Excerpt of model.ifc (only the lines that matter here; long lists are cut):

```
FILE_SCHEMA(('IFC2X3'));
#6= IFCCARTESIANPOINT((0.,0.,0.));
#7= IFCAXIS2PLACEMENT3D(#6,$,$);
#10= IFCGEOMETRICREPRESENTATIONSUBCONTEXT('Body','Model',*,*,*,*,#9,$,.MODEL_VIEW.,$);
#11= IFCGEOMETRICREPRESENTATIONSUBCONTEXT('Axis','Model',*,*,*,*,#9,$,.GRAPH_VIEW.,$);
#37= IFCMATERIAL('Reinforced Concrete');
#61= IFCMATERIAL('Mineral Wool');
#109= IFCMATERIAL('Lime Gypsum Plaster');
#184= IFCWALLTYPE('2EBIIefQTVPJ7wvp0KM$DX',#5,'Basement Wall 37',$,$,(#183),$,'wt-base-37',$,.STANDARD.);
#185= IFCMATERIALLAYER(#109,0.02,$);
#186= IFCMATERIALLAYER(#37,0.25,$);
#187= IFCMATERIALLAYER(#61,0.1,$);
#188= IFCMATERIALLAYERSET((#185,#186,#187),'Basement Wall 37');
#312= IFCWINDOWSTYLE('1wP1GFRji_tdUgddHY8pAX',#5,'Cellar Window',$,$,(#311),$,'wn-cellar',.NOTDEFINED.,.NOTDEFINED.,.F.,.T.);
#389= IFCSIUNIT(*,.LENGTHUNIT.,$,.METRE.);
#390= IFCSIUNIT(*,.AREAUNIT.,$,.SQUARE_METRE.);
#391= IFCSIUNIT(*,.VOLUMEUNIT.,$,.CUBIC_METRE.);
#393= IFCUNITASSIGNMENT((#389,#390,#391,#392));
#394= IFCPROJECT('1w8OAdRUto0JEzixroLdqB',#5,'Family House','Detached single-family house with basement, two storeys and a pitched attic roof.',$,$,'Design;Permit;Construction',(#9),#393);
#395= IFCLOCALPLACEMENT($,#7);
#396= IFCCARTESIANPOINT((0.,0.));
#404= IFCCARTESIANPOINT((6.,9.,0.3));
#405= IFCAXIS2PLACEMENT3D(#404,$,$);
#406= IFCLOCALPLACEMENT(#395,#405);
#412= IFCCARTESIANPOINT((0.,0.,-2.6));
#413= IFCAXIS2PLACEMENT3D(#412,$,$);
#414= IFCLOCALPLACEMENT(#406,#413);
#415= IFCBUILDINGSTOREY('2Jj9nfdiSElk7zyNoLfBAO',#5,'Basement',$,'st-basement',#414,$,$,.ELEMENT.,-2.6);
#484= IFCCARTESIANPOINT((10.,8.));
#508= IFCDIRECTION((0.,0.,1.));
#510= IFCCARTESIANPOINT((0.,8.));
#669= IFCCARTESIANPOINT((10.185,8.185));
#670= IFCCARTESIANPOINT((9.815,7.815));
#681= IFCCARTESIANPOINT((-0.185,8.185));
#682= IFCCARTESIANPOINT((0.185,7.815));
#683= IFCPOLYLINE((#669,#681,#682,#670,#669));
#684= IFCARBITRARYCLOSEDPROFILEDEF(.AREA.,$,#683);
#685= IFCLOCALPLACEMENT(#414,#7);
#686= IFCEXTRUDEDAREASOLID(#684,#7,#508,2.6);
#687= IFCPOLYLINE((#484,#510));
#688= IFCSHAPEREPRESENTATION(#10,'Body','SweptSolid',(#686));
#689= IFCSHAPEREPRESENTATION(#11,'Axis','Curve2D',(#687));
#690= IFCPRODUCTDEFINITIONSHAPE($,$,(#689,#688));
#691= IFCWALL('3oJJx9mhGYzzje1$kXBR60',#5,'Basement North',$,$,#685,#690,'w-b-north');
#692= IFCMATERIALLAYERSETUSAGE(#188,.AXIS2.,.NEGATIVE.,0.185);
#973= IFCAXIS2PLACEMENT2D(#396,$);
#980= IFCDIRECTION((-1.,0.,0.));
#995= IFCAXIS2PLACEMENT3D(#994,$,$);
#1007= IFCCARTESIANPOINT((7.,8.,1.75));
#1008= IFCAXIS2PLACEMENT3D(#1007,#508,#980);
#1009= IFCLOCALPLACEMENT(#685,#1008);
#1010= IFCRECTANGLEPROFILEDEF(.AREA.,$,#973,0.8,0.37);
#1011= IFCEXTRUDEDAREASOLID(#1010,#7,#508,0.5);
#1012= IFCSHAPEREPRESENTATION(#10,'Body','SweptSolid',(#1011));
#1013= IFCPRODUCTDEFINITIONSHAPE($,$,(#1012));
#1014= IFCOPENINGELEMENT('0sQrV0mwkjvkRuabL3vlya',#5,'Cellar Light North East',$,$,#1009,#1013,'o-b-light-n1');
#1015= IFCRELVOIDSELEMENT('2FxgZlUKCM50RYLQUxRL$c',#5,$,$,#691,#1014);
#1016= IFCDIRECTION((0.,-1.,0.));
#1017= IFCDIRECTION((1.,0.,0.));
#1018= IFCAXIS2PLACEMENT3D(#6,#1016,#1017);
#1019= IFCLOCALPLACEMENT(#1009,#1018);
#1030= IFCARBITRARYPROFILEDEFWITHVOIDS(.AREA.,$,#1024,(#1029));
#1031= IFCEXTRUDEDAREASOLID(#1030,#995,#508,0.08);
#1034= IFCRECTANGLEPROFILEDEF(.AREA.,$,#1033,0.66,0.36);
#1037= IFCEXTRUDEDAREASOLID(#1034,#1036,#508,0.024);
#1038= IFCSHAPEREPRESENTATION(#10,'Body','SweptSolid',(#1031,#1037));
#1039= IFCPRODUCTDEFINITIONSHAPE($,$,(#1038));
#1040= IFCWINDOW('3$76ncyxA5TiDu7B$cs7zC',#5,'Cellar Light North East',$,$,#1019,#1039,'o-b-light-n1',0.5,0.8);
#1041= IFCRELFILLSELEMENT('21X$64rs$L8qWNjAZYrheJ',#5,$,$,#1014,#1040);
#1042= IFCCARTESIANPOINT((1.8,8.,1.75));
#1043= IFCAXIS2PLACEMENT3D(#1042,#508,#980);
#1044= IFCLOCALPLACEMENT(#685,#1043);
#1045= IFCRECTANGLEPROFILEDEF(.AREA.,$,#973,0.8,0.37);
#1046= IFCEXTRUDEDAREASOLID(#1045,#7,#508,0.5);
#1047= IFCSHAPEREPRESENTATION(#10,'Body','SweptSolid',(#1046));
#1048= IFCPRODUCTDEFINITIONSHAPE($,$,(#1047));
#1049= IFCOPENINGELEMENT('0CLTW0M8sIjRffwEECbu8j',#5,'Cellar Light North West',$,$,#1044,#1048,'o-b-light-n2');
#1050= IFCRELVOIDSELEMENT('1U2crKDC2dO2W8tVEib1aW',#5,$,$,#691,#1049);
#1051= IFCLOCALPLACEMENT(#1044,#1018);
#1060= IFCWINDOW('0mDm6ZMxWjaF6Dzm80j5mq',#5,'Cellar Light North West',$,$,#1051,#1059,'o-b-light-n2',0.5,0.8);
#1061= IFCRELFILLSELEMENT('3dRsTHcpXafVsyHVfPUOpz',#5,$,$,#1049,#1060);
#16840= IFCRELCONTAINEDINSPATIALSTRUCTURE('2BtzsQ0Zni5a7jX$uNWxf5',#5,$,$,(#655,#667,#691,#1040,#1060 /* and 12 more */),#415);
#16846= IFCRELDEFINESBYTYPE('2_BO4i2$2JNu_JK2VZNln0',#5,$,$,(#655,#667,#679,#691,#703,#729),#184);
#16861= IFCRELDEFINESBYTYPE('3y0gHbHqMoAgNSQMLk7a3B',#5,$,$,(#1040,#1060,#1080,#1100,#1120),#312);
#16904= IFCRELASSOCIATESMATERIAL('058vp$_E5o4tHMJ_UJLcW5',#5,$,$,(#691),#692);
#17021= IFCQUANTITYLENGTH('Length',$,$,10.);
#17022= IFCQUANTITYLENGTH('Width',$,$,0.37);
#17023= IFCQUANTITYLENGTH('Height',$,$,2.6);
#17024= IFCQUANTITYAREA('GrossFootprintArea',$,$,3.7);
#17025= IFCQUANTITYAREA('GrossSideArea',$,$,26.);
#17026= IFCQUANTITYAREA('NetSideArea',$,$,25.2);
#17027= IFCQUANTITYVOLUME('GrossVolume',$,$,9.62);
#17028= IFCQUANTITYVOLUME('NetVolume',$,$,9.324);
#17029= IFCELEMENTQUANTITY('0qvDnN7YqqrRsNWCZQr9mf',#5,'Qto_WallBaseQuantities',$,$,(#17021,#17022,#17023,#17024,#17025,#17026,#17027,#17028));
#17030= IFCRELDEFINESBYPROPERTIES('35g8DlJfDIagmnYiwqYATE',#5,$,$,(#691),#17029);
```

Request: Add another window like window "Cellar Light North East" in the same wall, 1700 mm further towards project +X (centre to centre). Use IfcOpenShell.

```python
import ifcopenshell
import ifcopenshell.api.feature
import ifcopenshell.api.geometry
import ifcopenshell.api.pset
import ifcopenshell.api.root
import ifcopenshell.geom
import ifcopenshell.util.element
import ifcopenshell.util.placement
import ifcopenshell.util.shape
import ifcopenshell.util.unit

model = ifcopenshell.open("model.ifc")
area_scale = ifcopenshell.util.unit.calculate_unit_scale(model, "AREAUNIT")
volume_scale = ifcopenshell.util.unit.calculate_unit_scale(model, "VOLUMEUNIT")
settings = ifcopenshell.geom.settings()


def volume(element):
    """Net volume in cubic metres, openings subtracted."""
    shape = ifcopenshell.geom.create_shape(settings, element)
    return ifcopenshell.util.shape.get_volume(shape.geometry)


def reuse_history(source, copy):
    """copy_class also copies each property set's owner history, people and application; keep the originals."""
    for rel in copy.IsDefinedBy:
        if rel.is_a("IfcRelDefinesByProperties") and (history := rel.RelatingPropertyDefinition.OwnerHistory):
            rel.RelatingPropertyDefinition.OwnerHistory = source.OwnerHistory
            ifcopenshell.util.element.remove_deep2(model, history)


window = model.by_guid("3$76ncyxA5TiDu7B$cs7zC")
opening = window.FillsVoids[0].RelatingOpeningElement
wall = opening.VoidsElements[0].RelatingBuildingElement
before = volume(wall)
shift = ifcopenshell.util.placement.get_local_placement(wall.ObjectPlacement)[:3, 0] * 1.7

# copy_class copies the void relationship, type, container and properties, but no geometry.
new_opening = ifcopenshell.api.root.copy_class(model, product=opening)
new_opening.Representation = ifcopenshell.util.element.copy_deep(
    model, opening.Representation, exclude=["IfcGeometricRepresentationContext", "IfcRepresentationMap"]
)
new_opening.Tag = None
new_window = ifcopenshell.api.root.copy_class(model, product=window)
new_window.Representation = ifcopenshell.util.element.copy_deep(
    model, window.Representation, exclude=["IfcGeometricRepresentationContext", "IfcRepresentationMap"]
)
new_window.Tag = None
reuse_history(window, new_window)
fills = ifcopenshell.api.feature.add_filling(model, opening=new_opening, element=new_window)
fills.OwnerHistory = new_window.OwnerHistory  # required in IFC2X3

for old, new in ((opening, new_opening), (window, new_window)):
    matrix = ifcopenshell.util.placement.get_local_placement(old.ObjectPlacement)
    matrix[:3, 3] += shift
    ifcopenshell.api.geometry.edit_object_placement(model, product=new, matrix=matrix, is_si=False)

after = volume(wall)
thickness = 0.37  # wall thickness in metres

# Update the wall's stored quantities.
qto = model.by_id(ifcopenshell.util.element.get_pset(wall, "Qto_WallBaseQuantities", should_inherit=False)["id"])
ifcopenshell.api.pset.edit_qto(model, qto=qto, properties={
    "NetSideArea": after / thickness / area_scale,
    "NetVolume": after / volume_scale,
})

print(f"wall volume {before:.3f} -> {after:.3f} m3")

model.write("model_v2.ifc")
```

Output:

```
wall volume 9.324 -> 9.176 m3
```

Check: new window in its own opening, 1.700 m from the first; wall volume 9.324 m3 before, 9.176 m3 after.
